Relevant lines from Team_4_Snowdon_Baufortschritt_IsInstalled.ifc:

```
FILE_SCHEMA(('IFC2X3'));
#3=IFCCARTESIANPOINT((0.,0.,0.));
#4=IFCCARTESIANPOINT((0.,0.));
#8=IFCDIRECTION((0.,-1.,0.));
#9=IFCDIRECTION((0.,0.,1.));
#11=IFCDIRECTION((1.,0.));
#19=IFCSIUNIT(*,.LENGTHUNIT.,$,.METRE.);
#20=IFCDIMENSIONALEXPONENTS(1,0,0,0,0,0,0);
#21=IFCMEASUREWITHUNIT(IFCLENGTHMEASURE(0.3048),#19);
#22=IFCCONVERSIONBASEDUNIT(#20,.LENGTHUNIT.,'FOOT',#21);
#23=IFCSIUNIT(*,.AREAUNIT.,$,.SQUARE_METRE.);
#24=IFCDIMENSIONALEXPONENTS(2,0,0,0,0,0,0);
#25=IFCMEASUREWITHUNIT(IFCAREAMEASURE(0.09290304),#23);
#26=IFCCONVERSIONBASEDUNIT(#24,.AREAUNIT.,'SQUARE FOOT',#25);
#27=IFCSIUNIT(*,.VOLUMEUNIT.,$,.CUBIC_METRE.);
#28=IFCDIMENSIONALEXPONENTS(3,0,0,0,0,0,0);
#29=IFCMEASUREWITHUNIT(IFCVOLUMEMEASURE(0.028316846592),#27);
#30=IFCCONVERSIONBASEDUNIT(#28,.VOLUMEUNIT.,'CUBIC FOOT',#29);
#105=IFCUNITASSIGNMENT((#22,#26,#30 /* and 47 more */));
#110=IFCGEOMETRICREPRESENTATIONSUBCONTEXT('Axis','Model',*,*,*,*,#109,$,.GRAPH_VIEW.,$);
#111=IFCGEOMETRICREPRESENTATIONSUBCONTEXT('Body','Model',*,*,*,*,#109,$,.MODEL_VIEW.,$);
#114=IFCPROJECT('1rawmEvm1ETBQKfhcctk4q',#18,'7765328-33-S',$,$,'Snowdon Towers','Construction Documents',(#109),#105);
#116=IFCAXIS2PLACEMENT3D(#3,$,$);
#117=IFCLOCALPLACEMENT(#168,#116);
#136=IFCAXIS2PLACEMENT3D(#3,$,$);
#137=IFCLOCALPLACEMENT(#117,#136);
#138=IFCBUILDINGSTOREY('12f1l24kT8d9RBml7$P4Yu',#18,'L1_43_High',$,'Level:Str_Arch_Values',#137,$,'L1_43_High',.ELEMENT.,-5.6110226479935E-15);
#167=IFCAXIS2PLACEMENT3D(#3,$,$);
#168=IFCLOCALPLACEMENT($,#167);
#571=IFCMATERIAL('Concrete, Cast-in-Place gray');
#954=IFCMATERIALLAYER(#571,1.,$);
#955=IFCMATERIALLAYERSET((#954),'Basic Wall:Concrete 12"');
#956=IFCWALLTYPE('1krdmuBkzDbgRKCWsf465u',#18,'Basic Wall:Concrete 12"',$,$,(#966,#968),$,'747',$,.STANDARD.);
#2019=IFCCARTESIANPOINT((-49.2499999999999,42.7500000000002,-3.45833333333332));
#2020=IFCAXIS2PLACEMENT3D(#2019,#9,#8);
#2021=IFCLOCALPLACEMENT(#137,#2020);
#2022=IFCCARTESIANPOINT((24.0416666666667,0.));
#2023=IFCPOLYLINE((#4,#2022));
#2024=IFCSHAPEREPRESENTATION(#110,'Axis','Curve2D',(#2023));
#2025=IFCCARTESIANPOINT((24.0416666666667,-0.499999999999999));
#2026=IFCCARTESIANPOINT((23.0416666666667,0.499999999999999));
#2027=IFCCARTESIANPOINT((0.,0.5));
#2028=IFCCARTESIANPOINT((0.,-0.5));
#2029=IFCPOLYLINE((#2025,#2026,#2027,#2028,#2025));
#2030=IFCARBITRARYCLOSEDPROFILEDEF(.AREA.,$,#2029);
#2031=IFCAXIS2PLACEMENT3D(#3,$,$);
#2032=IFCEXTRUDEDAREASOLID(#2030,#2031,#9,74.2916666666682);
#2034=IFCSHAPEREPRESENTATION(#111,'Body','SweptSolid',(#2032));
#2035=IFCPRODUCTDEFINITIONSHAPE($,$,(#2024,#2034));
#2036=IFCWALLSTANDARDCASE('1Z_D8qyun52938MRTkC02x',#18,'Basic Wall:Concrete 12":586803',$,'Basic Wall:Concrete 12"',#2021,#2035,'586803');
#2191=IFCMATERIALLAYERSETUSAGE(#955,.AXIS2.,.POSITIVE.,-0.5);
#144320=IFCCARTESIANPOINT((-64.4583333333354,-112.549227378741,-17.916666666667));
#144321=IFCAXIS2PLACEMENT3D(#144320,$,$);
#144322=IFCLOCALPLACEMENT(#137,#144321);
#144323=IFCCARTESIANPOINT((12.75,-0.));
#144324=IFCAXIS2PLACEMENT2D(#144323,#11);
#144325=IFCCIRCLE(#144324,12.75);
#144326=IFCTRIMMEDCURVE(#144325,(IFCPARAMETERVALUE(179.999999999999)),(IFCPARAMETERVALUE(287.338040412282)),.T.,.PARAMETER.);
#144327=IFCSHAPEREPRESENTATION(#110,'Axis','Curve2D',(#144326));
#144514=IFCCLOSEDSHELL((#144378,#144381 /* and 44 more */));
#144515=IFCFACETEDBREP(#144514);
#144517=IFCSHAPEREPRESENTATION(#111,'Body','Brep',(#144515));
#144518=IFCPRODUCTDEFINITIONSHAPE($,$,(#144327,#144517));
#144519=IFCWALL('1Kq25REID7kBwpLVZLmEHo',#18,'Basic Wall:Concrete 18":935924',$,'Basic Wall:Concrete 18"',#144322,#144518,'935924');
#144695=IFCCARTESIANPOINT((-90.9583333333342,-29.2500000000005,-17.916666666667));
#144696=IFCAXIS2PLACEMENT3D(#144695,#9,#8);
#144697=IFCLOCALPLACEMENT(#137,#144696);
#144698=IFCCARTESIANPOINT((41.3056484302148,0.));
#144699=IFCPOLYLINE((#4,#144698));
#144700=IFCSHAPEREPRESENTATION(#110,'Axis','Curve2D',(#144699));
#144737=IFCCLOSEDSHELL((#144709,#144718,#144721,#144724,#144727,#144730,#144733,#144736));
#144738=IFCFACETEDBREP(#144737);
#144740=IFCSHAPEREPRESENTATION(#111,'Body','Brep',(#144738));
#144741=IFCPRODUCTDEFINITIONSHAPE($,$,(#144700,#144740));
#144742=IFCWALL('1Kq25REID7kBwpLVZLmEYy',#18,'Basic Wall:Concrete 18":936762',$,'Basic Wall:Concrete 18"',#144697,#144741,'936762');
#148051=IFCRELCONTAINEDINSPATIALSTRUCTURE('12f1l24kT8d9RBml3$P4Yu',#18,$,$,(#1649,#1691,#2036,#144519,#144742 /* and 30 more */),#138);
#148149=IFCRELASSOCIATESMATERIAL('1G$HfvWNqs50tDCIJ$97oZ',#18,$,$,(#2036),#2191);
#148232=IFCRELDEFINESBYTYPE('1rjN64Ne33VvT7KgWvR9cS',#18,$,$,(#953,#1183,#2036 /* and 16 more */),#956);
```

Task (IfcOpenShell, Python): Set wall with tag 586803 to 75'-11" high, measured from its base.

```python
import ifcopenshell
import ifcopenshell.geom
import ifcopenshell.util.representation
import ifcopenshell.util.shape
import ifcopenshell.util.unit

model = ifcopenshell.open("Team_4_Snowdon_Baufortschritt_IsInstalled.ifc")
unit_scale = ifcopenshell.util.unit.calculate_unit_scale(model)
settings = ifcopenshell.geom.settings()


def volume(element):
    """Net volume in cubic metres, openings subtracted."""
    shape = ifcopenshell.geom.create_shape(settings, element)
    return ifcopenshell.util.shape.get_volume(shape.geometry)


wall = model.by_id(2036)
before = volume(wall)

body = ifcopenshell.util.representation.get_representation(wall, "Model", "Body")
solid = body.Items[0]
old_height = solid.Depth
solid.Depth = 911 * 0.0254 / unit_scale
after = volume(wall)

print(f"height {old_height:g} -> {solid.Depth:g}, volume {before:.3f} -> {after:.3f} m3")

model.write("Team_4_Snowdon_Baufortschritt_IsInstalled_v2.ifc")
```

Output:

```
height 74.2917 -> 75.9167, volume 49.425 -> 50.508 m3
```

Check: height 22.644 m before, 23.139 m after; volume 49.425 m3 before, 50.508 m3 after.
